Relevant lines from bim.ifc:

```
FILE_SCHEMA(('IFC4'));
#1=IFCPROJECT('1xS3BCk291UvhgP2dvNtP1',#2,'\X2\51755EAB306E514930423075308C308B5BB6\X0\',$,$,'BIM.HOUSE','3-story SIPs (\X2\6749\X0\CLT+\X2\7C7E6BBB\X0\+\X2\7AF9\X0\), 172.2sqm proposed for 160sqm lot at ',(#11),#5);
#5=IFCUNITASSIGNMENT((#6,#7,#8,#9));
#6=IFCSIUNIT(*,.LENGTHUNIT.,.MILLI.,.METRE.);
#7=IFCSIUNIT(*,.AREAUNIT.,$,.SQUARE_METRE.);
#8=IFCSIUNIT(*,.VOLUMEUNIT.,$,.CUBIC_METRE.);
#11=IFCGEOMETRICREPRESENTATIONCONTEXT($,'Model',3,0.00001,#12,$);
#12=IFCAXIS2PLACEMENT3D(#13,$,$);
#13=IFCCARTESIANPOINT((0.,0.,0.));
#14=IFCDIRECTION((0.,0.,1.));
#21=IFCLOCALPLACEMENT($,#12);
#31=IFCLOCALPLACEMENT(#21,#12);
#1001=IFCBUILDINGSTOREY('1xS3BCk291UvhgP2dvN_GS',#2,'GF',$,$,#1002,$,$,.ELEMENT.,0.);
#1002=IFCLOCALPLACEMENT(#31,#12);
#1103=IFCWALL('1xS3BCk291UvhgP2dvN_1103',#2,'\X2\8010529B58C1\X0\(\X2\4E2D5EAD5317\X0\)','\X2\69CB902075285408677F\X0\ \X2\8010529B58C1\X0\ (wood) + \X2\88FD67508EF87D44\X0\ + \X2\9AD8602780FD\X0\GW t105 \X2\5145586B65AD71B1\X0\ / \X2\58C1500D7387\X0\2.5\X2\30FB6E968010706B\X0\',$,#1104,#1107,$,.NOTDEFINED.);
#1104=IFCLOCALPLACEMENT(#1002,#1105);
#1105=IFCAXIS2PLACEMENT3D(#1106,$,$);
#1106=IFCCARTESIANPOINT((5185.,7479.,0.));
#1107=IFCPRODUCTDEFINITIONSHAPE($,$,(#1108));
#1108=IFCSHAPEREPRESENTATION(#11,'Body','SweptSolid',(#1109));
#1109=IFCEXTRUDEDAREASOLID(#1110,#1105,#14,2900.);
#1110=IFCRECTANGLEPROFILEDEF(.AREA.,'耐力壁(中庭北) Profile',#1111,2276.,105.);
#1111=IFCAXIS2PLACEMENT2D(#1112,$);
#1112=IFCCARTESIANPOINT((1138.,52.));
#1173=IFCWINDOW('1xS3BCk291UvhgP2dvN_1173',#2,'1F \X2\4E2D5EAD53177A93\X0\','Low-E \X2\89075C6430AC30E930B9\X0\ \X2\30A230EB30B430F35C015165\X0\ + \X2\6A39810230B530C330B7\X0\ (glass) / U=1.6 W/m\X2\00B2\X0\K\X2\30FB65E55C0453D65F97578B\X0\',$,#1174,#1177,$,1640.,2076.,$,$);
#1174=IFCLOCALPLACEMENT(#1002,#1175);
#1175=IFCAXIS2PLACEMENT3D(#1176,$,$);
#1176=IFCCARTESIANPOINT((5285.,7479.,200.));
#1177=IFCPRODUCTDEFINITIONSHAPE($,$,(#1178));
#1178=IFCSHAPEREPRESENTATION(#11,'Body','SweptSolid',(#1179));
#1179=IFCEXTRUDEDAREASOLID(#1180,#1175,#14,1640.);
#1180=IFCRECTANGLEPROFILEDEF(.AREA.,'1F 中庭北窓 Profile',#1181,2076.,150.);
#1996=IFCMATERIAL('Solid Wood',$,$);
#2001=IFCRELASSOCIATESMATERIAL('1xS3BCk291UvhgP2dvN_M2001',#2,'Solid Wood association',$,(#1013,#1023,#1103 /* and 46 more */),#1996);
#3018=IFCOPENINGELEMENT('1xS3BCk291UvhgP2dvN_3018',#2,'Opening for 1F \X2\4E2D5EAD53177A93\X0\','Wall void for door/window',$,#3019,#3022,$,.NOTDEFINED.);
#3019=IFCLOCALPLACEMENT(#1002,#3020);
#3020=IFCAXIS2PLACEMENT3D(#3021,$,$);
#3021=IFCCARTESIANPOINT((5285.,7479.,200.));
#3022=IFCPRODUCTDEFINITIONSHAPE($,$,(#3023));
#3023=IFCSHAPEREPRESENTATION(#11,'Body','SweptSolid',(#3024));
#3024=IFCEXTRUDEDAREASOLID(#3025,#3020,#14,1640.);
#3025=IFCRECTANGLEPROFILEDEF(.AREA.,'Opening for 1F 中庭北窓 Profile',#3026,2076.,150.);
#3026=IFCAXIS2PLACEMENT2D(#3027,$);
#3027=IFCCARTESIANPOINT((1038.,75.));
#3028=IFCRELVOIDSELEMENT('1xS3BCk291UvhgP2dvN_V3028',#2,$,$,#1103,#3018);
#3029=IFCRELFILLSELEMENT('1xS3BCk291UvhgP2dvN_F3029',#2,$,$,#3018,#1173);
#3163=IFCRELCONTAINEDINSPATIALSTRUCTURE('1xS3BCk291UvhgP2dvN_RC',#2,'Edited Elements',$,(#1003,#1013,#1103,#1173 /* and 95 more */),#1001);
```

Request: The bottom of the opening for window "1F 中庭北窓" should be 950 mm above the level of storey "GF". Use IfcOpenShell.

```python
import numpy as np
import ifcopenshell
import ifcopenshell.api.geometry
import ifcopenshell.geom
import ifcopenshell.util.element
import ifcopenshell.util.placement
import ifcopenshell.util.shape
import ifcopenshell.util.unit

model = ifcopenshell.open("bim.ifc")
unit_scale = ifcopenshell.util.unit.calculate_unit_scale(model)

window = model.by_id(1173)
opening = window.FillsVoids[0].RelatingOpeningElement
storey = ifcopenshell.util.element.get_container(window, ifc_class="IfcBuildingStorey")
level = ifcopenshell.util.placement.get_local_placement(storey.ObjectPlacement)[2, 3]

# The opening's origin need not be at the sill, so measure its lowest point.
shape = ifcopenshell.geom.create_shape(ifcopenshell.geom.settings(), opening)
bottom = ifcopenshell.util.shape.get_shape_bottom_elevation(shape, shape.geometry) / unit_scale
dz = level + 0.95 / unit_scale - bottom

shift = np.array([0.0, 0.0, dz])
# The window is not placed relative to its opening, so move both.
for product in (opening, window):
    matrix = ifcopenshell.util.placement.get_local_placement(product.ObjectPlacement)
    matrix[:3, 3] += shift
    ifcopenshell.api.geometry.edit_object_placement(model, product=product, matrix=matrix, is_si=False)

print(f"moved by {dz * unit_scale:+.3f} m")

model.write("bim-out.ifc")
```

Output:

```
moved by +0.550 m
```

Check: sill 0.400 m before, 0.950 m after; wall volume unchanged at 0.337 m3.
